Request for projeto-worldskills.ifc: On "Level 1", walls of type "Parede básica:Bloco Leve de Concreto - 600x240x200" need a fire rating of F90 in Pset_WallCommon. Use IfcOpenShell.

First a look at what the model holds.

```python
import ifcopenshell
import ifcopenshell.util.element

model = ifcopenshell.open("projeto-worldskills.ifc")
print(model.schema)
storey = next(s for s in model.by_type("IfcBuildingStorey") if s.Name == "Level 1")
walls = [e for e in ifcopenshell.util.element.get_decomposition(storey) if e.is_a("IfcWall")]
seen = {}
for e in walls:
    element_type = ifcopenshell.util.element.get_type(e)
    key = (element_type.Name if element_type != e and element_type else None, ifcopenshell.util.element.get_pset(e, "Pset_WallCommon", "FireRating"))
    seen[key] = seen.get(key, 0) + 1
for (name, value), count in sorted(seen.items(), key=str):
    print(count, "x", name, "|", value)
```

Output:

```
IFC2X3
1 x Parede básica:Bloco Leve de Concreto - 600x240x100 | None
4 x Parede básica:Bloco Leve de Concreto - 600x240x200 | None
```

```python
import ifcopenshell
import ifcopenshell.api.pset
import ifcopenshell.util.element

model = ifcopenshell.open("projeto-worldskills.ifc")

storey = next(s for s in model.by_type("IfcBuildingStorey") if s.Name == "Level 1")
walls = [e for e in ifcopenshell.util.element.get_decomposition(storey) if e.is_a("IfcWall")]

count = 0
for e in walls:
    element_type = ifcopenshell.util.element.get_type(e)
    if element_type in (None, e) or element_type.Name != "Parede básica:Bloco Leve de Concreto - 600x240x200":
        continue
    # add_pset returns the element's existing set when there is one.
    pset = ifcopenshell.api.pset.add_pset(model, product=e, name="Pset_WallCommon")
    ifcopenshell.api.pset.edit_pset(model, pset=pset, properties={"FireRating": "F90"})
    count += 1

print(count, "walls updated")

model.write("projeto-worldskills_rev.ifc")
```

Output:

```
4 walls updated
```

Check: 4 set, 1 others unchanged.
